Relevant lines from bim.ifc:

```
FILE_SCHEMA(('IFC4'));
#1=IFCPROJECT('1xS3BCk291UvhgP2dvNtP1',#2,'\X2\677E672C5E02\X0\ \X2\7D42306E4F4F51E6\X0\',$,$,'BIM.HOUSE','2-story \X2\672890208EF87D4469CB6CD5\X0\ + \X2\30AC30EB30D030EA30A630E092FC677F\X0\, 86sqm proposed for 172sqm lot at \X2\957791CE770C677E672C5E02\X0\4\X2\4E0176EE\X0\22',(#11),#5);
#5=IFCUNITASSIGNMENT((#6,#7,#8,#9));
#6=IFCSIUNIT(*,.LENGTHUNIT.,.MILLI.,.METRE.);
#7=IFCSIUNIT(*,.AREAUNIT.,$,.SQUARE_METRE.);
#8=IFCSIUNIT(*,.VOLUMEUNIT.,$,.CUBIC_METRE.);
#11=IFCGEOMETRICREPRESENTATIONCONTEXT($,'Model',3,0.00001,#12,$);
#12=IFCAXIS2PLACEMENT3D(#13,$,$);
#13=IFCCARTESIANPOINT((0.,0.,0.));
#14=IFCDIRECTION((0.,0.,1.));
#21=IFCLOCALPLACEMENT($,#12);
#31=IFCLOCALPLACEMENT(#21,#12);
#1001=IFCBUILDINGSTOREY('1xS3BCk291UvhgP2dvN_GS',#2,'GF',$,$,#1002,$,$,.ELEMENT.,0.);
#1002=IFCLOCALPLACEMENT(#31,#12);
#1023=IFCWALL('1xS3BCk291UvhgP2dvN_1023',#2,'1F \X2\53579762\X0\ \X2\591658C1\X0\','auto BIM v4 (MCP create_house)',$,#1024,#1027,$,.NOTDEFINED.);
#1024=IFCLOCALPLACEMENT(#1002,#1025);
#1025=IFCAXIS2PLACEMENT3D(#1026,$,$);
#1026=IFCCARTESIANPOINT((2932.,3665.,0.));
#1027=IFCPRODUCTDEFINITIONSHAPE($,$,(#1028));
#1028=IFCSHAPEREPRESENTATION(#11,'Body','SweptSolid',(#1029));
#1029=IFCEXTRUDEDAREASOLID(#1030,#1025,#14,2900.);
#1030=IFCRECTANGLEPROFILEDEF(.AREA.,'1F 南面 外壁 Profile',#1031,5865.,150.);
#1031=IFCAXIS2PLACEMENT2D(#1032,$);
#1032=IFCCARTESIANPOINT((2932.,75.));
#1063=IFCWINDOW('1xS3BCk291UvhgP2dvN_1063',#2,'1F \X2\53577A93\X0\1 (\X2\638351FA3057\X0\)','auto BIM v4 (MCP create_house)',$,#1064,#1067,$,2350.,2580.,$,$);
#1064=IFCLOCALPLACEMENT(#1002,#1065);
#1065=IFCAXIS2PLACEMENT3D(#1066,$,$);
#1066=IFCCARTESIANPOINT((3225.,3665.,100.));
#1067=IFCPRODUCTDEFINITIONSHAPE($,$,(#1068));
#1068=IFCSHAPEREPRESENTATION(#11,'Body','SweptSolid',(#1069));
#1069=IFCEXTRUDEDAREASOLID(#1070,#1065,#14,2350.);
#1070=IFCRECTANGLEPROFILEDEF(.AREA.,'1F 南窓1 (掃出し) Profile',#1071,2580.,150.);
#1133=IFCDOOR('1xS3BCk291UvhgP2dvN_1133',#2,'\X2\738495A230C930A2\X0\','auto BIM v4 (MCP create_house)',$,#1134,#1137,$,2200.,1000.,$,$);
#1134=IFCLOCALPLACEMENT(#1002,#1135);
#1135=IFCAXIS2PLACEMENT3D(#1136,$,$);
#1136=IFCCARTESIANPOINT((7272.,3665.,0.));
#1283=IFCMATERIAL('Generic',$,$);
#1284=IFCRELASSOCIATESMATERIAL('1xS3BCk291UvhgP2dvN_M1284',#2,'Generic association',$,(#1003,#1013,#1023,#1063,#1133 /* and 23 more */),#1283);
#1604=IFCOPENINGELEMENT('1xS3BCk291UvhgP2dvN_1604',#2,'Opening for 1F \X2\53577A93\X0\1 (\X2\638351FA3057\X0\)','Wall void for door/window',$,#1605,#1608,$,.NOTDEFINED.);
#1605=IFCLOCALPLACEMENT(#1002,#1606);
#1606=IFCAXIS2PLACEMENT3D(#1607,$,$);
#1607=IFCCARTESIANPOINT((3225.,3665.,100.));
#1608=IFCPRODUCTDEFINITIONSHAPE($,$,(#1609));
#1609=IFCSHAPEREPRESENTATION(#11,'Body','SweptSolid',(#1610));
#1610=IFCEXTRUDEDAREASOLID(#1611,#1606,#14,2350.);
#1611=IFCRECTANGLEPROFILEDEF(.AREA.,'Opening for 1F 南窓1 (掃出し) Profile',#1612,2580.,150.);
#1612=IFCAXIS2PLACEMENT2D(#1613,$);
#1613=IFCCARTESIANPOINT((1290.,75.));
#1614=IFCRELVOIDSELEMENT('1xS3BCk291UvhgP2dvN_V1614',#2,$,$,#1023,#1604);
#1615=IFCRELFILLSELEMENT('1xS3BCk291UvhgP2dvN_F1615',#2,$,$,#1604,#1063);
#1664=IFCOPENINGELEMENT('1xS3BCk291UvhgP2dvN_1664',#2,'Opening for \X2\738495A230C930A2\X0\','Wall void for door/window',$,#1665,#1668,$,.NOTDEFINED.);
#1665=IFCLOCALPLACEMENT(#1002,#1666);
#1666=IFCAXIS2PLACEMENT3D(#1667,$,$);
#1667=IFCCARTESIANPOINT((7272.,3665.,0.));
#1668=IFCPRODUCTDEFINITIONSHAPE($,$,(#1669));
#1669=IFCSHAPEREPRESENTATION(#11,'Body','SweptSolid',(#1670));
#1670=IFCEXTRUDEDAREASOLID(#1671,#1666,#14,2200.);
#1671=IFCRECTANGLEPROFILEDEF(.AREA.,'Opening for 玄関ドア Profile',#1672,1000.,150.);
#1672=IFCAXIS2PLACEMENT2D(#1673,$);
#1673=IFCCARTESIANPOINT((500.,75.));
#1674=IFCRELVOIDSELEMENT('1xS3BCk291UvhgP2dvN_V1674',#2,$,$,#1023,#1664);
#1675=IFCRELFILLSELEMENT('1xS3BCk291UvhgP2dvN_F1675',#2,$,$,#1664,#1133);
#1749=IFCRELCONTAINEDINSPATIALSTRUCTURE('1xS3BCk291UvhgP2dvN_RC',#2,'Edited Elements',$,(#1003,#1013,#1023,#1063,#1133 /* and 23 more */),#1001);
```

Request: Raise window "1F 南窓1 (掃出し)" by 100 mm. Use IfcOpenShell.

```python
import numpy as np
import ifcopenshell
import ifcopenshell.api.geometry
import ifcopenshell.util.placement
import ifcopenshell.util.unit

model = ifcopenshell.open("bim.ifc")
unit_scale = ifcopenshell.util.unit.calculate_unit_scale(model)

window = model.by_id(1063)
opening = window.FillsVoids[0].RelatingOpeningElement
dz = 0.1 / unit_scale

shift = np.array([0.0, 0.0, dz])
# The window is not placed relative to its opening, so move both.
for product in (opening, window):
    matrix = ifcopenshell.util.placement.get_local_placement(product.ObjectPlacement)
    matrix[:3, 3] += shift
    ifcopenshell.api.geometry.edit_object_placement(model, product=product, matrix=matrix, is_si=False)

print(f"moved by {dz * unit_scale:+.3f} m")

model.write("bim_rev.ifc")
```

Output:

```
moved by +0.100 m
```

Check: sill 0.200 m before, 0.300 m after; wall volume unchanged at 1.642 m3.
